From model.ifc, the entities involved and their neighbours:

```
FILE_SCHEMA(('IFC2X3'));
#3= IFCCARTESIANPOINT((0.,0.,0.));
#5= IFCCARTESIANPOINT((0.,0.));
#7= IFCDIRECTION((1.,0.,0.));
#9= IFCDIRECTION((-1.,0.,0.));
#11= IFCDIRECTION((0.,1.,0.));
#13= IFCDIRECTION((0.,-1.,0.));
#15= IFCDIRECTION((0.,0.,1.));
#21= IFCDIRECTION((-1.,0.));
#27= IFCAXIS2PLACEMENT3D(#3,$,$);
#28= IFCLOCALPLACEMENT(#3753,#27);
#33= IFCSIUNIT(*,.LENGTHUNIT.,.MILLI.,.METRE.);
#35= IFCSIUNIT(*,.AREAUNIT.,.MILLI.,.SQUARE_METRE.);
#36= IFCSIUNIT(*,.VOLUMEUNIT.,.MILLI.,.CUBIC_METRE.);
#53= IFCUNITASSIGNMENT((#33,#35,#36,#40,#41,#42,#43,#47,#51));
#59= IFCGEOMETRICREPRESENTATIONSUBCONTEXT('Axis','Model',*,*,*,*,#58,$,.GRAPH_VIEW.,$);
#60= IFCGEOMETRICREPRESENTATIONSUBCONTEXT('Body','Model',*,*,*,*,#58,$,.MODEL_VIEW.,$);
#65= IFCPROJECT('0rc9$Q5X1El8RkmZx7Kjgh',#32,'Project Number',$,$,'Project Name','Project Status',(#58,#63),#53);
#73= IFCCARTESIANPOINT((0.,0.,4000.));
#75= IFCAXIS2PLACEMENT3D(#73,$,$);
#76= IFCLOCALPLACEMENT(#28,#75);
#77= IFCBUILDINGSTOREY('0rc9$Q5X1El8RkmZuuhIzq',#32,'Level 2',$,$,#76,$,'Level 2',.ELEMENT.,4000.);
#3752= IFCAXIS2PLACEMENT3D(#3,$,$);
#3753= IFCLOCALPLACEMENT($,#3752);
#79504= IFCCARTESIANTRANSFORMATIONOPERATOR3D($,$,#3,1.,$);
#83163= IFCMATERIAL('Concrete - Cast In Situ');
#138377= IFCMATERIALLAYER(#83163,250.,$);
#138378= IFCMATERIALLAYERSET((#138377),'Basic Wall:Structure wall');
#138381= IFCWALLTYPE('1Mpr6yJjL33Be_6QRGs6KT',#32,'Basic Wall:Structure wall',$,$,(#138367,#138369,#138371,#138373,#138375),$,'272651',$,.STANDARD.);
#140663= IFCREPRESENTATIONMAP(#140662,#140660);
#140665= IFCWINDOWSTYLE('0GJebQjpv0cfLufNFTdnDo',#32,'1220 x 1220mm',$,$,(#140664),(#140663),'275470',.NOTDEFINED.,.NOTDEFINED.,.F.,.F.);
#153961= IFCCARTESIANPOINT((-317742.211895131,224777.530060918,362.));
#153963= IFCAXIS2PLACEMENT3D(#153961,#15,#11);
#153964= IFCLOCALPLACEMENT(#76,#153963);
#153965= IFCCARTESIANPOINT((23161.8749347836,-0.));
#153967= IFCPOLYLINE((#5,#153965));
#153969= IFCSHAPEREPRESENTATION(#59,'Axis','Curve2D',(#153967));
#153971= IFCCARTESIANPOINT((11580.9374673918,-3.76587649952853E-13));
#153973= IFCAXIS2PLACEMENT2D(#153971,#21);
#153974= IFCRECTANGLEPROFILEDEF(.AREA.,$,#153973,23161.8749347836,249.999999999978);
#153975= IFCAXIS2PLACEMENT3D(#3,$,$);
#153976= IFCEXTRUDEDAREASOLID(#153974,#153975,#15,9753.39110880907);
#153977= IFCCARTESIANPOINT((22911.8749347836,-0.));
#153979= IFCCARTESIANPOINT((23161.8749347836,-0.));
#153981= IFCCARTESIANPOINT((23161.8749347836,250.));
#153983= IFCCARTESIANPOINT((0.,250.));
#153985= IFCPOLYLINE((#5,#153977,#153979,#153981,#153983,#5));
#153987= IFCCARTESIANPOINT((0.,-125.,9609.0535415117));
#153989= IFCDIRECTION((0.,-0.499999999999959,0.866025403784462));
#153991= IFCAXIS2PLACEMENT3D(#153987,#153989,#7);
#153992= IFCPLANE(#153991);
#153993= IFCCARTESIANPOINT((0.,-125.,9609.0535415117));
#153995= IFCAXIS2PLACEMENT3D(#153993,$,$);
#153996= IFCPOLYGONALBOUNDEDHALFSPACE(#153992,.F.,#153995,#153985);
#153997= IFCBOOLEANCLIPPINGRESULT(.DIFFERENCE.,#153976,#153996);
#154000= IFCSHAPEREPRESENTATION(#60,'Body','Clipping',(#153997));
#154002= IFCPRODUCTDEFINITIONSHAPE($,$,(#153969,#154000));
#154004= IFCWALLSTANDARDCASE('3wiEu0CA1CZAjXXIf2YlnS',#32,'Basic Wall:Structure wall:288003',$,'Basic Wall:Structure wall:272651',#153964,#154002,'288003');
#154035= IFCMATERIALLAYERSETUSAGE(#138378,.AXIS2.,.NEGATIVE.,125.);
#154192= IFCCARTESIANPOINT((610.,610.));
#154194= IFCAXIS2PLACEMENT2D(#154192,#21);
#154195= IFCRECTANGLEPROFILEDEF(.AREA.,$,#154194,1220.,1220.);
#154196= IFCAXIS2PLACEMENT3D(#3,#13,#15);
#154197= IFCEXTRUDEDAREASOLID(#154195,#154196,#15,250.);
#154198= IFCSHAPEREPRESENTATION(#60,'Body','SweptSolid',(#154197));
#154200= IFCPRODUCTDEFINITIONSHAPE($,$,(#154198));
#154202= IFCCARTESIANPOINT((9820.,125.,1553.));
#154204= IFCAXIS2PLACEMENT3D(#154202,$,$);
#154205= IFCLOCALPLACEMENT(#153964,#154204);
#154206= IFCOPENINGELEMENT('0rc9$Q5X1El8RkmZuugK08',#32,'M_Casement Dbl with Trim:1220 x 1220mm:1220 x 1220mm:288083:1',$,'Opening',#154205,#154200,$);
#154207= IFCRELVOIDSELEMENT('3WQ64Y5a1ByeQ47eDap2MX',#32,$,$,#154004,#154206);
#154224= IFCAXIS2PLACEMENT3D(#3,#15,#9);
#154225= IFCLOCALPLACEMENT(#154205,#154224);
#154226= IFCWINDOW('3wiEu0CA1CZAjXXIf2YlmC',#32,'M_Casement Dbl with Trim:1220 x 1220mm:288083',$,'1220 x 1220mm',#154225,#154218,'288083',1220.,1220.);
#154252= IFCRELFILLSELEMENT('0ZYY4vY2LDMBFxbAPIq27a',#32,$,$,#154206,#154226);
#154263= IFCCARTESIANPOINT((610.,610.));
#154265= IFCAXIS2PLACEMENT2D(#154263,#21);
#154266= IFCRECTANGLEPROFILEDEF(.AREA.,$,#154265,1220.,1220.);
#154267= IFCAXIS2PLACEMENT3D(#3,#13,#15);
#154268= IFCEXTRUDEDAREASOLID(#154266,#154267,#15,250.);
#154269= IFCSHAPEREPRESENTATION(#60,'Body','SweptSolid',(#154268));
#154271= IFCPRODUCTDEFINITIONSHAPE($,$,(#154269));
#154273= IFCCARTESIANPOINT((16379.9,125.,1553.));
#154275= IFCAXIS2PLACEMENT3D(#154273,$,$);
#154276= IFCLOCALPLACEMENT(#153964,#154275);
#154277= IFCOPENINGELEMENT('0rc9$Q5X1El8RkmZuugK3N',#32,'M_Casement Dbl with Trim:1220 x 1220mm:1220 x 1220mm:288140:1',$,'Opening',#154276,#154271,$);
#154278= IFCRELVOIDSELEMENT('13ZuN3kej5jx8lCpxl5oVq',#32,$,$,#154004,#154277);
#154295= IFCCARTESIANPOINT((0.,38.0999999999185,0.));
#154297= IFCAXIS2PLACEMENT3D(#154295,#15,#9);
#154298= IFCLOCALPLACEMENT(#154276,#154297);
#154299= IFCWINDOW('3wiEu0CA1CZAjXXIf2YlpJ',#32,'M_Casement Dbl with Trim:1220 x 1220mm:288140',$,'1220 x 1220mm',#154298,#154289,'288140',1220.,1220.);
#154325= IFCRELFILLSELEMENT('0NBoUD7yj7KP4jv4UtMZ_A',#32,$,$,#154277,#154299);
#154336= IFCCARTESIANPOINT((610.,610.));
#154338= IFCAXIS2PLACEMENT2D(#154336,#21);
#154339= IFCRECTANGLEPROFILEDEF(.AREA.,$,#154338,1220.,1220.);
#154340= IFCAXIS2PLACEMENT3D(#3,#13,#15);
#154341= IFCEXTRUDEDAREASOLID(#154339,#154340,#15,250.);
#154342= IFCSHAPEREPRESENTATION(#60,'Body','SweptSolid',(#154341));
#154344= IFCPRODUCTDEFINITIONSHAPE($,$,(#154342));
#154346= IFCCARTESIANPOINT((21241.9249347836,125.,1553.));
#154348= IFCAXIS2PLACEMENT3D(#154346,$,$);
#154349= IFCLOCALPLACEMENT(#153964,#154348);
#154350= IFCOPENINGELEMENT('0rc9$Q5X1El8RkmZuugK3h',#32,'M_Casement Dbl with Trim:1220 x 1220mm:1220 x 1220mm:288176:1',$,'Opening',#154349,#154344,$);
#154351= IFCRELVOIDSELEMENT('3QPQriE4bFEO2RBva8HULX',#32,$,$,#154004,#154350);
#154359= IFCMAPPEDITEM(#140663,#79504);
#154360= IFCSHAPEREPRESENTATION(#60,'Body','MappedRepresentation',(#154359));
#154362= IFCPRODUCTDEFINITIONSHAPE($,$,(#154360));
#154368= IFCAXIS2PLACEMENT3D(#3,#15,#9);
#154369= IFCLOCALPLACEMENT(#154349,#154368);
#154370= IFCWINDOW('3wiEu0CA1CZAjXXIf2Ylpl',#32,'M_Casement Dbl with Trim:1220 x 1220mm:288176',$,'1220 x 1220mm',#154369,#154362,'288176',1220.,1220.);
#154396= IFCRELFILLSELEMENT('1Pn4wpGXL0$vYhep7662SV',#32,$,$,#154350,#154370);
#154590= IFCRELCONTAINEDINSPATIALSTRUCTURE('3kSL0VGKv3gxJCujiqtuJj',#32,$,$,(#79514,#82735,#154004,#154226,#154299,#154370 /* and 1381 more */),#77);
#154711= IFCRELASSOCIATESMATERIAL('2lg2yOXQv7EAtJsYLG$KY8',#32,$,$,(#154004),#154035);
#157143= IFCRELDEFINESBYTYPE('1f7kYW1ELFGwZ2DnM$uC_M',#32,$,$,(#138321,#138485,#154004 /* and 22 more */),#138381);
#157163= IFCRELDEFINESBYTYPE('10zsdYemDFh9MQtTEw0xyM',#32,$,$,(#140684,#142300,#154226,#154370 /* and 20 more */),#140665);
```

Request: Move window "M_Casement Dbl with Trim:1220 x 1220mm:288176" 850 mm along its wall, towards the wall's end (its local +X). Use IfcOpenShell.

```python
import ifcopenshell
import ifcopenshell.api.geometry
import ifcopenshell.util.placement
import ifcopenshell.util.unit

model = ifcopenshell.open("model.ifc")
unit_scale = ifcopenshell.util.unit.calculate_unit_scale(model)

window = model.by_id(154370)
opening = window.FillsVoids[0].RelatingOpeningElement
wall = opening.VoidsElements[0].RelatingBuildingElement

wall_matrix = ifcopenshell.util.placement.get_local_placement(wall.ObjectPlacement)
shift = wall_matrix[:3, 0] * 0.85 / unit_scale
before = ifcopenshell.util.placement.get_local_placement(window.ObjectPlacement)[:3, 3].copy()

# The window is placed relative to its opening, so it follows when the opening moves.
matrix = ifcopenshell.util.placement.get_local_placement(opening.ObjectPlacement)
matrix[:3, 3] += shift
ifcopenshell.api.geometry.edit_object_placement(
    model, product=opening, matrix=matrix, is_si=False, should_transform_children=True
)

after = ifcopenshell.util.placement.get_local_placement(window.ObjectPlacement)[:3, 3]
print("window moved by", (after - before).round(3) + 0.0)

model.write("model-out.ifc")
```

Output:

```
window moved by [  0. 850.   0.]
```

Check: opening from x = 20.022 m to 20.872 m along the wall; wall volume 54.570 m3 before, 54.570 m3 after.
